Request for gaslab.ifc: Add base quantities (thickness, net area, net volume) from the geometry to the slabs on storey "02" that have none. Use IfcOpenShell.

First a look at what the model holds.

```python
import ifcopenshell
import ifcopenshell.util.element
import ifcopenshell.util.unit

model = ifcopenshell.open("gaslab.ifc")
print(model.schema)
for unit_type in ("LENGTHUNIT", "AREAUNIT", "VOLUMEUNIT"):
    print(unit_type, ifcopenshell.util.unit.calculate_unit_scale(model, unit_type))
storey = next(s for s in model.by_type("IfcBuildingStorey") if s.Name == "02")
slabs = [e for e in ifcopenshell.util.element.get_decomposition(storey) if e.is_a("IfcSlab")]
for e in sorted(slabs, key=lambda e: e.id()):
    print(e.id(), e.is_a(), e.Name, list(ifcopenshell.util.element.get_psets(e, qtos_only=True)), sep=" | ")
```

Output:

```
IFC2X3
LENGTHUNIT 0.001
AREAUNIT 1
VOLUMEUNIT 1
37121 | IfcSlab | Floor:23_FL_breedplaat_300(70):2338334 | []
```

```python
import ifcopenshell
import ifcopenshell.api.pset
import ifcopenshell.geom
import ifcopenshell.util.element
import ifcopenshell.util.shape
import ifcopenshell.util.unit

model = ifcopenshell.open("gaslab.ifc")
unit_scale = ifcopenshell.util.unit.calculate_unit_scale(model)
area_scale = ifcopenshell.util.unit.calculate_unit_scale(model, "AREAUNIT")
volume_scale = ifcopenshell.util.unit.calculate_unit_scale(model, "VOLUMEUNIT")
settings = ifcopenshell.geom.settings()

storey = next(s for s in model.by_type("IfcBuildingStorey") if s.Name == "02")
slabs = [e for e in ifcopenshell.util.element.get_decomposition(storey) if e.is_a("IfcSlab")]

for e in sorted(slabs, key=lambda e: e.id()):
    if ifcopenshell.util.element.get_psets(e, qtos_only=True, should_inherit=False):
        continue
    # Geometry comes back in metres, in the element's own axes.
    shape = ifcopenshell.geom.create_shape(settings, e)
    values = {
        "Width": ifcopenshell.util.shape.get_z(shape.geometry) / unit_scale,
        "NetArea": ifcopenshell.util.shape.get_footprint_area(shape.geometry) / area_scale,
        "NetVolume": ifcopenshell.util.shape.get_volume(shape.geometry) / volume_scale,
    }
    qto = ifcopenshell.api.pset.add_qto(model, product=e, name="BaseQuantities")
    ifcopenshell.api.pset.edit_qto(model, qto=qto, properties=values)
    print(e.id(), {k: round(v, 3) for k, v in values.items()})

model.write("gaslab_edited.ifc")
```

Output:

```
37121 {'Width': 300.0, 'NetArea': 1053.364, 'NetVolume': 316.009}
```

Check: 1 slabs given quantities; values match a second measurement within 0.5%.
